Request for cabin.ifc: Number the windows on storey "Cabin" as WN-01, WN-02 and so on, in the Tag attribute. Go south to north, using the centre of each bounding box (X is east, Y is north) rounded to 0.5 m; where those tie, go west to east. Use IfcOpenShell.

First a look at what the model holds.

```python
import ifcopenshell
import ifcopenshell.util.element
import ifcopenshell.util.placement

model = ifcopenshell.open("cabin.ifc")
print(model.schema)
storey = next(s for s in model.by_type("IfcBuildingStorey") if s.Name == "Cabin")
windows = [e for e in ifcopenshell.util.element.get_decomposition(storey) if e.is_a("IfcWindow")]
for e in sorted(windows, key=lambda e: e.id()):
    origin = ifcopenshell.util.placement.get_local_placement(e.ObjectPlacement)[:3, 3]
    print(e.id(), e.Tag, e.Name, origin.round(2) + 0.0, sep=" | ")
```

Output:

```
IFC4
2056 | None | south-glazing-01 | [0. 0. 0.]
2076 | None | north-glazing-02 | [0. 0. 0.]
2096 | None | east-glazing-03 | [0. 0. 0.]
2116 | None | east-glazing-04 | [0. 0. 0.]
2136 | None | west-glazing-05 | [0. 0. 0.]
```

```python
import ifcopenshell
import ifcopenshell.geom
import ifcopenshell.util.element
import ifcopenshell.util.shape

model = ifcopenshell.open("cabin.ifc")
settings = ifcopenshell.geom.settings()
settings.set("use-world-coords", True)


def centre(element):
    shape = ifcopenshell.geom.create_shape(settings, element)
    return ifcopenshell.util.shape.get_bbox_centroid(shape.geometry)


storey = next(s for s in model.by_type("IfcBuildingStorey") if s.Name == "Cabin")
windows = [e for e in ifcopenshell.util.element.get_decomposition(storey) if e.is_a("IfcWindow")]

# Insertion points can sit at a corner or the storey origin, so sort by the geometry (in metres).
centres = {e: centre(e) for e in windows}
windows.sort(key=lambda e: (round(centres[e][1] / 0.5), centres[e][0]))

for i, e in enumerate(windows, start=1):
    number = f"WN-{i:02d}"
    e.Tag = number
    print(e.id(), number)

model.write("cabin_edited.ifc")
```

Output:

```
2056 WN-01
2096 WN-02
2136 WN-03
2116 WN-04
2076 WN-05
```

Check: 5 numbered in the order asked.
